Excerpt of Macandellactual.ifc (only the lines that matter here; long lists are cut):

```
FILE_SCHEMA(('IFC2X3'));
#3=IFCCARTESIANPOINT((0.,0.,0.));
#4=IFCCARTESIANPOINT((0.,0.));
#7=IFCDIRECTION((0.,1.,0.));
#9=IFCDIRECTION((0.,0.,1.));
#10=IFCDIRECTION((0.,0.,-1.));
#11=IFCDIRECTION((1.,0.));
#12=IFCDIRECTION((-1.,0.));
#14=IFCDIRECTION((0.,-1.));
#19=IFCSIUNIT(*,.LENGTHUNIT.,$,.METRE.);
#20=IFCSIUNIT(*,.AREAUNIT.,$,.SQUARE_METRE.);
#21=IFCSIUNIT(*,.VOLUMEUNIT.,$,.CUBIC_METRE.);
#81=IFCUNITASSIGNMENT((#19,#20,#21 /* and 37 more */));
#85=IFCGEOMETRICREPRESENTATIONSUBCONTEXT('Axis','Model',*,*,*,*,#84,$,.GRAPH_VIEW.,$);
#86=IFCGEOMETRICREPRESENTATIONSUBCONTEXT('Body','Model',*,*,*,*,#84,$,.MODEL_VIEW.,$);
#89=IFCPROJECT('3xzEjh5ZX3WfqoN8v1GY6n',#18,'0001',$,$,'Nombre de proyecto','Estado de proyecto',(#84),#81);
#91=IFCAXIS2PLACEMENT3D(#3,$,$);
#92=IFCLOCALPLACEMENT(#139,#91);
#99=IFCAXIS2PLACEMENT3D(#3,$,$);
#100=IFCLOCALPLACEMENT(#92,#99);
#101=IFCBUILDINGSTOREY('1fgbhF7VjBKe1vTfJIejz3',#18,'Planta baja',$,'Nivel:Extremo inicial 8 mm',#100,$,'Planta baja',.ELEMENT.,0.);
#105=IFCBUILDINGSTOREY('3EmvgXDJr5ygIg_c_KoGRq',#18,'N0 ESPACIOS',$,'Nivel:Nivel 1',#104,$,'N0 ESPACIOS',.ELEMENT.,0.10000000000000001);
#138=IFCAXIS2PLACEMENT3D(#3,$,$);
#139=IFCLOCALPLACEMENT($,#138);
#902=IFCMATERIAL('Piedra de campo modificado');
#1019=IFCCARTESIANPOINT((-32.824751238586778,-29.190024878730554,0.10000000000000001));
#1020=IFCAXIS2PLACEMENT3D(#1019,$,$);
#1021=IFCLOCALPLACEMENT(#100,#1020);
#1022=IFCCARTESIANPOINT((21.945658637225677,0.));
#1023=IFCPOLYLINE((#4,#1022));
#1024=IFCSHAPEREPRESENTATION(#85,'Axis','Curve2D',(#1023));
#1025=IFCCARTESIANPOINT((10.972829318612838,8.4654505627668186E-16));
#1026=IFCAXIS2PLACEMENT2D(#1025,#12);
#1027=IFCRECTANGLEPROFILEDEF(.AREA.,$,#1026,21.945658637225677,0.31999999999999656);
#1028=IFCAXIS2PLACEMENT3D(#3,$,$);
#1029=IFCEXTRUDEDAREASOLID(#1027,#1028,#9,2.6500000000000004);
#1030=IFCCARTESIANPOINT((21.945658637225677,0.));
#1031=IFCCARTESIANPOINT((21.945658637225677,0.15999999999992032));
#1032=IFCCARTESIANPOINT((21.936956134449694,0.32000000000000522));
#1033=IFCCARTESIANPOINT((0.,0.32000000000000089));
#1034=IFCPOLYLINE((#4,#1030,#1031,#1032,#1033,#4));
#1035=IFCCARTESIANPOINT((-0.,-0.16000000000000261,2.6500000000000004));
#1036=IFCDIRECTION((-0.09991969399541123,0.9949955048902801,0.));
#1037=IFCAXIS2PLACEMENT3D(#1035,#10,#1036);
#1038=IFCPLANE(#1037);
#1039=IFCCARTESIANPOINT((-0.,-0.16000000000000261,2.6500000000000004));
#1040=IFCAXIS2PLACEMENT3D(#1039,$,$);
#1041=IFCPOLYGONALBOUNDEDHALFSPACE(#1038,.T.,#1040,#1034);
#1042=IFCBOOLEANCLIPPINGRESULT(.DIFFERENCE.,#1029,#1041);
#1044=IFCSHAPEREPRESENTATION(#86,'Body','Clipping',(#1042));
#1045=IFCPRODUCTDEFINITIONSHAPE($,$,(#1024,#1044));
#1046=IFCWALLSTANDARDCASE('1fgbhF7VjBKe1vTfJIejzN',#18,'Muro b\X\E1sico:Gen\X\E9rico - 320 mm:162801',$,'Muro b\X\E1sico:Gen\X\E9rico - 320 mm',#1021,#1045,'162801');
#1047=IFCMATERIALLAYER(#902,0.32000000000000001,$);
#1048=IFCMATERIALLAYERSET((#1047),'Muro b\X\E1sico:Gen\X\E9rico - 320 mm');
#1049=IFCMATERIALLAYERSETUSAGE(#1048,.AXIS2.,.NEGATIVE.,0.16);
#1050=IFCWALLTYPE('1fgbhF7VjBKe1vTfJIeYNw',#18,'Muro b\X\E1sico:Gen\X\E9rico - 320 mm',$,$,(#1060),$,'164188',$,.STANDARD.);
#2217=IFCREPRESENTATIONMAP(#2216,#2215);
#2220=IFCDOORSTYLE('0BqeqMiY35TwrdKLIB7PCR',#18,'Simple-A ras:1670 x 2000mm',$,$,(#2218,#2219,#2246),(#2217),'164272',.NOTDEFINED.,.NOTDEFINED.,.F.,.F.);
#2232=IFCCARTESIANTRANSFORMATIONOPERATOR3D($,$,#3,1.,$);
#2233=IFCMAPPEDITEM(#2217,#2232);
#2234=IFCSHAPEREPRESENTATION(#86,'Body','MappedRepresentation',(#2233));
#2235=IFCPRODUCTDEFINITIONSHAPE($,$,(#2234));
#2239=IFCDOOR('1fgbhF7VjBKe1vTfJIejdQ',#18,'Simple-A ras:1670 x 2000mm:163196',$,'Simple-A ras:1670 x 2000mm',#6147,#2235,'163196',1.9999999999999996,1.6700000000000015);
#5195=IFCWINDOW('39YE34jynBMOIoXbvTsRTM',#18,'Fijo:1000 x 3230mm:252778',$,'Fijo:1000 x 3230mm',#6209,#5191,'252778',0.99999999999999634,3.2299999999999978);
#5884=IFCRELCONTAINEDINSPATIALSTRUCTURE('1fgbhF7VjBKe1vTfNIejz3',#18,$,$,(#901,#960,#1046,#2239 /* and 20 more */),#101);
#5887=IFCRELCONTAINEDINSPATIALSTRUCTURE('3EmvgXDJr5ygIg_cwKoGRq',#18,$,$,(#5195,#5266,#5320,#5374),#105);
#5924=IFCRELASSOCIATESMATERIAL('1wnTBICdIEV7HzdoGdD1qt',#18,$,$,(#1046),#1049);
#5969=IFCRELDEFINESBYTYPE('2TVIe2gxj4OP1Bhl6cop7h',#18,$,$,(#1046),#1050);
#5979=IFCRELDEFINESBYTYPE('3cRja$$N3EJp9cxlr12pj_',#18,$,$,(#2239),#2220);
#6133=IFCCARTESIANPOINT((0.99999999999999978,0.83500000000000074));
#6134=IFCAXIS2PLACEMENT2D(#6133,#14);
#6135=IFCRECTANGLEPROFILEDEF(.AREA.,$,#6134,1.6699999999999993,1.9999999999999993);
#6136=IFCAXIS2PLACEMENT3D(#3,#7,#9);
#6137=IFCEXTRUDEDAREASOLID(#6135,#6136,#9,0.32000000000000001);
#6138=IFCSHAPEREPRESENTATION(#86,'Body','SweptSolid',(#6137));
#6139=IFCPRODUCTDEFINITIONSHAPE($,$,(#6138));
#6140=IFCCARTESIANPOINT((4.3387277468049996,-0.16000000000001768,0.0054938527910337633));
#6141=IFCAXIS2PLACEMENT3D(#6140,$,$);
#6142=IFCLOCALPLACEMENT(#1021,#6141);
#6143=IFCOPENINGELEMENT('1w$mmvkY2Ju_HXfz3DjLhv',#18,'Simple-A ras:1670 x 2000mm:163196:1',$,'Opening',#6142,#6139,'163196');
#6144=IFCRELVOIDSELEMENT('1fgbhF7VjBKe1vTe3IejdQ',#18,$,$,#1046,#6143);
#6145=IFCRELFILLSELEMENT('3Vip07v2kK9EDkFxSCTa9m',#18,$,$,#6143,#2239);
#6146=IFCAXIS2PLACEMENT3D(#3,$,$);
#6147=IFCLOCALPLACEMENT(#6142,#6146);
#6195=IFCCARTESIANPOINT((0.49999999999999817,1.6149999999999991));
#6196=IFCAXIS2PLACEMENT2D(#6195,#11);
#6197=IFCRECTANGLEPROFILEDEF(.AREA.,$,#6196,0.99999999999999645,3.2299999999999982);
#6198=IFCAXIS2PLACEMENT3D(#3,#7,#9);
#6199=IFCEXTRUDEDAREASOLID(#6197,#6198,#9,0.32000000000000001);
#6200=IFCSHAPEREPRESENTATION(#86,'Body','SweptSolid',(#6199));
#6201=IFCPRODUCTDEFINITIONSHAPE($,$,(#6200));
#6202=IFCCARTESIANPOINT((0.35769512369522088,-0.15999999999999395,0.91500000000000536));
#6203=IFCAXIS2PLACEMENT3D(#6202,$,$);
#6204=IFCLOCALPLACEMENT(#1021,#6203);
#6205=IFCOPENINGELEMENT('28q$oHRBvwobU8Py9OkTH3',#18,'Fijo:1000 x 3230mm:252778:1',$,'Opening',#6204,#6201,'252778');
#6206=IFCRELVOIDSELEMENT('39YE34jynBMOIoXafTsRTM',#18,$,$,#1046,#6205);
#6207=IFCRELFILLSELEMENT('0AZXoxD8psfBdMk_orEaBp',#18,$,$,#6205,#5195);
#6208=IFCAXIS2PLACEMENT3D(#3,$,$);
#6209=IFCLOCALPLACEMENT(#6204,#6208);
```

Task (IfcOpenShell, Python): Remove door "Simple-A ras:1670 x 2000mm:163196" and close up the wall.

```python
import ifcopenshell
import ifcopenshell.api.feature
import ifcopenshell.api.root
import ifcopenshell.geom
import ifcopenshell.util.shape

model = ifcopenshell.open("Macandellactual.ifc")
settings = ifcopenshell.geom.settings()


def volume(element):
    """Net volume in cubic metres, openings subtracted."""
    shape = ifcopenshell.geom.create_shape(settings, element)
    return ifcopenshell.util.shape.get_volume(shape.geometry)


door = model.by_guid("1fgbhF7VjBKe1vTfJIejdQ")
opening = door.FillsVoids[0].RelatingOpeningElement
wall = opening.VoidsElements[0].RelatingBuildingElement
before = volume(wall)

ifcopenshell.api.root.remove_product(model, product=door)
ifcopenshell.api.feature.remove_feature(model, feature=opening)

after = volume(wall)

print(f"wall volume {before:.3f} -> {after:.3f} m3")

model.write("Macandellactual_v2.ifc")
```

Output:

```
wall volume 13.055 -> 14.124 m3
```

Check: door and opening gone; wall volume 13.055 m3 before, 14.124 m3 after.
